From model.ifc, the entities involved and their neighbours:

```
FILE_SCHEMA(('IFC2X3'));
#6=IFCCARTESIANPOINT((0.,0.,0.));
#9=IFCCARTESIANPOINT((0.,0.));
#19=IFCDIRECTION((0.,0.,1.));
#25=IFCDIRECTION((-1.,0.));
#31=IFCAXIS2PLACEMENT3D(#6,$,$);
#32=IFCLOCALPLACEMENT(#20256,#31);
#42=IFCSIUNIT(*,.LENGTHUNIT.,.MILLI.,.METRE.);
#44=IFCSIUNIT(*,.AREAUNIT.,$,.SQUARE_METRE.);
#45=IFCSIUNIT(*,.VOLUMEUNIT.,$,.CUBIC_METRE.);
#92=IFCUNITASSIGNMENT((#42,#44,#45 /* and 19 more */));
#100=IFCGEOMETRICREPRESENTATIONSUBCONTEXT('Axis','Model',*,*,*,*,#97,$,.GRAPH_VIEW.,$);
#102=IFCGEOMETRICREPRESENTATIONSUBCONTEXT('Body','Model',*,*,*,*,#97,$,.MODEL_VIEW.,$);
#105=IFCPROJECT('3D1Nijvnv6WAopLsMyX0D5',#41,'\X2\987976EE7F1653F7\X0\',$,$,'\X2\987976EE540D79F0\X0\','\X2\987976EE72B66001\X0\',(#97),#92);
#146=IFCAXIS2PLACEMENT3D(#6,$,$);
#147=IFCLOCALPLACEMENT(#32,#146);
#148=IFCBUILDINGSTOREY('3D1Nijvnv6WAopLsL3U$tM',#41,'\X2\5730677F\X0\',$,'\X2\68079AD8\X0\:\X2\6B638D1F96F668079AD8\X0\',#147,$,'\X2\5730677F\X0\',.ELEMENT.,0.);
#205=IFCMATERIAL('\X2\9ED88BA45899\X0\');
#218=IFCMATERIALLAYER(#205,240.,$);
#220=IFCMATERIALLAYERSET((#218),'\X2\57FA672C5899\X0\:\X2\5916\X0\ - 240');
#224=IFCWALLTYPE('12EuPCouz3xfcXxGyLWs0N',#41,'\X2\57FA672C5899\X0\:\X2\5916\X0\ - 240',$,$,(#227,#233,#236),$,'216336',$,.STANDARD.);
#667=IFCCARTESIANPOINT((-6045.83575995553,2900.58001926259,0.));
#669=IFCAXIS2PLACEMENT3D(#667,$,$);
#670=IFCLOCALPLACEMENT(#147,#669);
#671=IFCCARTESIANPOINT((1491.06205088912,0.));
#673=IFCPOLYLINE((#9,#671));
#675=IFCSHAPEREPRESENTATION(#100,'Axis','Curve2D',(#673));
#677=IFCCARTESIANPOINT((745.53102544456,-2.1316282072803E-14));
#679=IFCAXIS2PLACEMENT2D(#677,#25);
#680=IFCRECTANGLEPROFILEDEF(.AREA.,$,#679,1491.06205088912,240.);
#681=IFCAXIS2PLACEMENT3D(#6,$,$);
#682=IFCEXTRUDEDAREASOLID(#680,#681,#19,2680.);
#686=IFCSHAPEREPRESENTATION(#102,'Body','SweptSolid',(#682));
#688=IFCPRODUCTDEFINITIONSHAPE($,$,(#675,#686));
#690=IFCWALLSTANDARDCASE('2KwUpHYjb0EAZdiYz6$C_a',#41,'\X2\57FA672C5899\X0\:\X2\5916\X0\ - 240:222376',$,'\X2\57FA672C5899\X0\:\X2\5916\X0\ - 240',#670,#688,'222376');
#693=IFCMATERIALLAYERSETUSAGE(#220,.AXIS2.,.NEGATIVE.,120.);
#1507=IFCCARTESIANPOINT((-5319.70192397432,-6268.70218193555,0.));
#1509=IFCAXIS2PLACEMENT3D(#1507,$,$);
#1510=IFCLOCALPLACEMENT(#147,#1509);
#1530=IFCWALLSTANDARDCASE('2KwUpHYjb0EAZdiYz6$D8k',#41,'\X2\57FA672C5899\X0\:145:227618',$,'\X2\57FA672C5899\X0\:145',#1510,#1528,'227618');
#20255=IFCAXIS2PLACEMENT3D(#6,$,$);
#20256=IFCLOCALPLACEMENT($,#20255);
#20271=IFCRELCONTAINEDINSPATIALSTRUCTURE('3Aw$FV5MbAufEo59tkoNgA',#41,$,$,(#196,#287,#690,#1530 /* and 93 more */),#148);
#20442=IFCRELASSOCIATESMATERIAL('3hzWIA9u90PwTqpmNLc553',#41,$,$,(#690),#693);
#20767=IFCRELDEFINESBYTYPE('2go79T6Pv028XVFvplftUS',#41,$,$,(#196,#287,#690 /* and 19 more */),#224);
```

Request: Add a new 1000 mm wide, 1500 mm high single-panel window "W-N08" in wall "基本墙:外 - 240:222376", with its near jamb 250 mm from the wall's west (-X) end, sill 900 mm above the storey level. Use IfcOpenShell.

```python
import numpy as np
import ifcopenshell
import ifcopenshell.api.feature
import ifcopenshell.api.geometry
import ifcopenshell.api.root
import ifcopenshell.api.spatial
import ifcopenshell.api.type
import ifcopenshell.geom
import ifcopenshell.util.element
import ifcopenshell.util.placement
import ifcopenshell.util.representation
import ifcopenshell.util.shape
import ifcopenshell.util.unit

model = ifcopenshell.open("model.ifc")
unit_scale = ifcopenshell.util.unit.calculate_unit_scale(model)
settings = ifcopenshell.geom.settings()


def volume(element):
    """Net volume in cubic metres, openings subtracted."""
    shape = ifcopenshell.geom.create_shape(settings, element)
    return ifcopenshell.util.shape.get_volume(shape.geometry)


wall = model.by_id(690)
storey = ifcopenshell.util.element.get_container(wall, ifc_class="IfcBuildingStorey")
context = ifcopenshell.util.representation.get_context(model, "Model", "Body", "MODEL_VIEW")
before = volume(wall)

width, height, from_end, sill = 1, 1.5, 0.25, 0.9  # metres

# The wall runs along its own X axis, and the end named is its -X end.
wall_shape = ifcopenshell.geom.create_shape(settings, wall)
x, y, z = ifcopenshell.util.shape.get_vertices(wall_shape.geometry).T
start = x.min() + from_end
face, thickness = float(y.min()), float(y.max() - y.min())
wall_matrix = ifcopenshell.util.placement.get_local_placement(wall.ObjectPlacement)
level = ifcopenshell.util.placement.get_local_placement(storey.ObjectPlacement)[2, 3]


def in_wall(x, y):
    """Placement at x, y metres in the wall's axes, at sill height."""
    matrix = wall_matrix.copy()
    matrix[:, 3] = wall_matrix @ np.array([x / unit_scale, y / unit_scale, 0.0, 1.0])
    matrix[2, 3] = level + sill / unit_scale
    return matrix


# Opening: a box that overshoots both wall faces by 50 mm.
opening = ifcopenshell.api.root.create_entity(model, ifc_class="IfcOpeningElement")
box = ifcopenshell.api.geometry.add_wall_representation(
    model, context=context, length=width, height=height, thickness=thickness + 0.1
)
ifcopenshell.api.geometry.assign_representation(model, product=opening, representation=box)
ifcopenshell.api.geometry.edit_object_placement(model, product=opening, matrix=in_wall(start, face - 0.05), is_si=False)
ifcopenshell.api.feature.add_feature(model, feature=opening, element=wall)

window = ifcopenshell.api.root.create_entity(model, ifc_class="IfcWindow", name="W-N08")
window.OverallWidth, window.OverallHeight = width / unit_scale, height / unit_scale
body = ifcopenshell.api.geometry.add_window_representation(
    model,
    context=context,
    overall_width=window.OverallWidth,
    overall_height=window.OverallHeight,
    partition_type="SINGLE_PANEL",
)
ifcopenshell.api.geometry.assign_representation(model, product=window, representation=body)
ifcopenshell.api.spatial.assign_container(model, products=[window], relating_structure=storey)
fills = ifcopenshell.api.feature.add_filling(model, opening=opening, element=window)
fills.OwnerHistory = window.OwnerHistory  # required in IFC2X3

# IFC2X3 keeps the operation on the window style.
style = ifcopenshell.api.root.create_entity(model, ifc_class="IfcWindowStyle", name="W-N08")
style.OperationType, style.ConstructionType = "SINGLE_PANEL", "NOTDEFINED"
style.ParameterTakesPrecedence = style.Sizeable = False
ifcopenshell.api.type.assign_type(model, related_objects=[window], relating_type=style)

# Centre the window in the wall's thickness.
ifcopenshell.api.geometry.edit_object_placement(model, product=window, matrix=in_wall(start, face), is_si=False)
window_shape = ifcopenshell.geom.create_shape(settings, window)
depth = ifcopenshell.util.shape.get_vertices(window_shape.geometry)[:, 1]
offset = face + thickness / 2 - (depth.min() + depth.max()) / 2
ifcopenshell.api.geometry.edit_object_placement(model, product=window, matrix=in_wall(start, offset), is_si=False)

after = volume(wall)

print(f"wall volume {before:.3f} -> {after:.3f} m3")

model.write("model_edited.ifc")
```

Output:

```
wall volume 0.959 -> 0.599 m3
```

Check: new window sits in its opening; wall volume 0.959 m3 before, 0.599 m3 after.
